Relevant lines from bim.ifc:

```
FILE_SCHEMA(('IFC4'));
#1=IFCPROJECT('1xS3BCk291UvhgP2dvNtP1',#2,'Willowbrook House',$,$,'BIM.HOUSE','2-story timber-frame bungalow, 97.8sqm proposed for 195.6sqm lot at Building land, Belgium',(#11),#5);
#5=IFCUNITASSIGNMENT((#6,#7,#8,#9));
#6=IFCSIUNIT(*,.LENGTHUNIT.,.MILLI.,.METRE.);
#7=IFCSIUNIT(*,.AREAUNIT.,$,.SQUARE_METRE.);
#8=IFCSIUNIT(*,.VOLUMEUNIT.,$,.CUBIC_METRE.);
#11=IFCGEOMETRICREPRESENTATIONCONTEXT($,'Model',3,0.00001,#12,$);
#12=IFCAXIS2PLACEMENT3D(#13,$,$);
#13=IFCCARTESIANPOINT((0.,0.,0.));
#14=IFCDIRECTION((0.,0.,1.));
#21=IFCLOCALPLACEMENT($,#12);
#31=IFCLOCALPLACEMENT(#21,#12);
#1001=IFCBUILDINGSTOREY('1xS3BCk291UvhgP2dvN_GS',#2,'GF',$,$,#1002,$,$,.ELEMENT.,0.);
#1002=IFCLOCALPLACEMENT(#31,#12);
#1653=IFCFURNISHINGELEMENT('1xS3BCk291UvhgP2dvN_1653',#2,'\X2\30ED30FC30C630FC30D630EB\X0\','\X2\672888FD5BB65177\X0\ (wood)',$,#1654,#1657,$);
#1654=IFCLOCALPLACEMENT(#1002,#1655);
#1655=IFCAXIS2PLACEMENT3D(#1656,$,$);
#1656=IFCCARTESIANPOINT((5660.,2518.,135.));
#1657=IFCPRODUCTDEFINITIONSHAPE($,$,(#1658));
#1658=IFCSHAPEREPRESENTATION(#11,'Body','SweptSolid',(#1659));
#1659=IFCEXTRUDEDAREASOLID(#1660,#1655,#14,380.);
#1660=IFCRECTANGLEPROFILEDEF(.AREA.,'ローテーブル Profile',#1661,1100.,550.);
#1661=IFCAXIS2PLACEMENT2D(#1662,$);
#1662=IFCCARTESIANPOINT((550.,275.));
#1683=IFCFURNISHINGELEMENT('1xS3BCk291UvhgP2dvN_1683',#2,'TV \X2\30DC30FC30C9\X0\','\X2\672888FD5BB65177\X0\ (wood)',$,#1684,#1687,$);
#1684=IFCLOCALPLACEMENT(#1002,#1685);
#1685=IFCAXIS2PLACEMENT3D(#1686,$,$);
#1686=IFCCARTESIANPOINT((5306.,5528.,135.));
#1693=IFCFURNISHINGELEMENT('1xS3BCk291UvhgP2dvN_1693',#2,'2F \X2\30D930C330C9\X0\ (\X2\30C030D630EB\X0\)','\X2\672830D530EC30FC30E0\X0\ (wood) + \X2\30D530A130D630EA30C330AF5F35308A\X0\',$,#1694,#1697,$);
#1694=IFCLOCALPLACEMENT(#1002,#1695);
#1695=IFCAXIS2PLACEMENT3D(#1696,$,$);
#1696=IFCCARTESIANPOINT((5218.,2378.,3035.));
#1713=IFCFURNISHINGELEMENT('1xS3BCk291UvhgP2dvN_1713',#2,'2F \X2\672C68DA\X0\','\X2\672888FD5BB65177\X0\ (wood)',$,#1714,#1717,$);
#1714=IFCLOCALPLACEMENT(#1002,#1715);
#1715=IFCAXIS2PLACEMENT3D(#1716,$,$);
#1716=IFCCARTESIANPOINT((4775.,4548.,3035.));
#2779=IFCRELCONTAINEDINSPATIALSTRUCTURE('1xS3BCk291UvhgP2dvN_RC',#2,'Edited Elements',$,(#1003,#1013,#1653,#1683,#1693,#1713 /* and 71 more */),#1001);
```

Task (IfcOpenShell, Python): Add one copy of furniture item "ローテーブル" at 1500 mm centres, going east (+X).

```python
import numpy as np
import ifcopenshell
import ifcopenshell.api.geometry
import ifcopenshell.api.root
import ifcopenshell.util.element
import ifcopenshell.util.placement

model = ifcopenshell.open("bim.ifc")


def reuse_history(source, copy):
    """copy_class also copies each property set's owner history, people and application; keep the originals."""
    for rel in copy.IsDefinedBy:
        if rel.is_a("IfcRelDefinesByProperties") and (history := rel.RelatingPropertyDefinition.OwnerHistory):
            rel.RelatingPropertyDefinition.OwnerHistory = source.OwnerHistory
            ifcopenshell.util.element.remove_deep2(model, history)


source = model.by_guid("1xS3BCk291UvhgP2dvN_1653")
base = ifcopenshell.util.placement.get_local_placement(source.ObjectPlacement)
step = np.array([1.0, 0.0, 0.0]) * 1500.0

for i in range(1, 2):
    copy = ifcopenshell.api.root.copy_class(model, product=source)
    copy.Representation = ifcopenshell.util.element.copy_deep(
        model, source.Representation, exclude=["IfcGeometricRepresentationContext", "IfcRepresentationMap"]
    )
    reuse_history(source, copy)
    matrix = base.copy()
    matrix[:3, 3] += i * step
    print("added at", matrix[:3, 3].round(3) + 0.0)
    ifcopenshell.api.geometry.edit_object_placement(model, product=copy, matrix=matrix, is_si=False)

model.write("bim_v2.ifc")
```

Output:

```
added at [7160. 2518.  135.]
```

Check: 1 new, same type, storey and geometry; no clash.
